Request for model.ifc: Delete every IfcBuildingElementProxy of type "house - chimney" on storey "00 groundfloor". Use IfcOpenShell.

First a look at what the model holds.

```python
import ifcopenshell
import ifcopenshell.util.element

model = ifcopenshell.open("model.ifc")
print(model.schema)
storey = next(s for s in model.by_type("IfcBuildingStorey") if s.Name == "00 groundfloor")
proxies = [e for e in ifcopenshell.util.element.get_decomposition(storey) if e.is_a("IfcBuildingElementProxy")]
seen = {}
for e in proxies:
    element_type = ifcopenshell.util.element.get_type(e)
    name = element_type.Name if element_type not in (None, e) else None
    seen[name] = seen.get(name, 0) + 1
for name, count in sorted(seen.items(), key=str):
    print(count, "x", name)
```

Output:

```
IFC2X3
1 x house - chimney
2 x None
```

```python
import ifcopenshell
import ifcopenshell.api.root
import ifcopenshell.util.element

model = ifcopenshell.open("model.ifc")

storey = next(s for s in model.by_type("IfcBuildingStorey") if s.Name == "00 groundfloor")
proxies = [e for e in ifcopenshell.util.element.get_decomposition(storey) if e.is_a("IfcBuildingElementProxy")]
targets = [e for e in proxies if (t := ifcopenshell.util.element.get_type(e)) not in (None, e) and t.Name == "house - chimney"]

for e in targets:
    ifcopenshell.api.root.remove_product(model, product=e)
print(len(targets), "removed")

model.write("model_updated.ifc")
```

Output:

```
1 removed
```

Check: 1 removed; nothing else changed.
